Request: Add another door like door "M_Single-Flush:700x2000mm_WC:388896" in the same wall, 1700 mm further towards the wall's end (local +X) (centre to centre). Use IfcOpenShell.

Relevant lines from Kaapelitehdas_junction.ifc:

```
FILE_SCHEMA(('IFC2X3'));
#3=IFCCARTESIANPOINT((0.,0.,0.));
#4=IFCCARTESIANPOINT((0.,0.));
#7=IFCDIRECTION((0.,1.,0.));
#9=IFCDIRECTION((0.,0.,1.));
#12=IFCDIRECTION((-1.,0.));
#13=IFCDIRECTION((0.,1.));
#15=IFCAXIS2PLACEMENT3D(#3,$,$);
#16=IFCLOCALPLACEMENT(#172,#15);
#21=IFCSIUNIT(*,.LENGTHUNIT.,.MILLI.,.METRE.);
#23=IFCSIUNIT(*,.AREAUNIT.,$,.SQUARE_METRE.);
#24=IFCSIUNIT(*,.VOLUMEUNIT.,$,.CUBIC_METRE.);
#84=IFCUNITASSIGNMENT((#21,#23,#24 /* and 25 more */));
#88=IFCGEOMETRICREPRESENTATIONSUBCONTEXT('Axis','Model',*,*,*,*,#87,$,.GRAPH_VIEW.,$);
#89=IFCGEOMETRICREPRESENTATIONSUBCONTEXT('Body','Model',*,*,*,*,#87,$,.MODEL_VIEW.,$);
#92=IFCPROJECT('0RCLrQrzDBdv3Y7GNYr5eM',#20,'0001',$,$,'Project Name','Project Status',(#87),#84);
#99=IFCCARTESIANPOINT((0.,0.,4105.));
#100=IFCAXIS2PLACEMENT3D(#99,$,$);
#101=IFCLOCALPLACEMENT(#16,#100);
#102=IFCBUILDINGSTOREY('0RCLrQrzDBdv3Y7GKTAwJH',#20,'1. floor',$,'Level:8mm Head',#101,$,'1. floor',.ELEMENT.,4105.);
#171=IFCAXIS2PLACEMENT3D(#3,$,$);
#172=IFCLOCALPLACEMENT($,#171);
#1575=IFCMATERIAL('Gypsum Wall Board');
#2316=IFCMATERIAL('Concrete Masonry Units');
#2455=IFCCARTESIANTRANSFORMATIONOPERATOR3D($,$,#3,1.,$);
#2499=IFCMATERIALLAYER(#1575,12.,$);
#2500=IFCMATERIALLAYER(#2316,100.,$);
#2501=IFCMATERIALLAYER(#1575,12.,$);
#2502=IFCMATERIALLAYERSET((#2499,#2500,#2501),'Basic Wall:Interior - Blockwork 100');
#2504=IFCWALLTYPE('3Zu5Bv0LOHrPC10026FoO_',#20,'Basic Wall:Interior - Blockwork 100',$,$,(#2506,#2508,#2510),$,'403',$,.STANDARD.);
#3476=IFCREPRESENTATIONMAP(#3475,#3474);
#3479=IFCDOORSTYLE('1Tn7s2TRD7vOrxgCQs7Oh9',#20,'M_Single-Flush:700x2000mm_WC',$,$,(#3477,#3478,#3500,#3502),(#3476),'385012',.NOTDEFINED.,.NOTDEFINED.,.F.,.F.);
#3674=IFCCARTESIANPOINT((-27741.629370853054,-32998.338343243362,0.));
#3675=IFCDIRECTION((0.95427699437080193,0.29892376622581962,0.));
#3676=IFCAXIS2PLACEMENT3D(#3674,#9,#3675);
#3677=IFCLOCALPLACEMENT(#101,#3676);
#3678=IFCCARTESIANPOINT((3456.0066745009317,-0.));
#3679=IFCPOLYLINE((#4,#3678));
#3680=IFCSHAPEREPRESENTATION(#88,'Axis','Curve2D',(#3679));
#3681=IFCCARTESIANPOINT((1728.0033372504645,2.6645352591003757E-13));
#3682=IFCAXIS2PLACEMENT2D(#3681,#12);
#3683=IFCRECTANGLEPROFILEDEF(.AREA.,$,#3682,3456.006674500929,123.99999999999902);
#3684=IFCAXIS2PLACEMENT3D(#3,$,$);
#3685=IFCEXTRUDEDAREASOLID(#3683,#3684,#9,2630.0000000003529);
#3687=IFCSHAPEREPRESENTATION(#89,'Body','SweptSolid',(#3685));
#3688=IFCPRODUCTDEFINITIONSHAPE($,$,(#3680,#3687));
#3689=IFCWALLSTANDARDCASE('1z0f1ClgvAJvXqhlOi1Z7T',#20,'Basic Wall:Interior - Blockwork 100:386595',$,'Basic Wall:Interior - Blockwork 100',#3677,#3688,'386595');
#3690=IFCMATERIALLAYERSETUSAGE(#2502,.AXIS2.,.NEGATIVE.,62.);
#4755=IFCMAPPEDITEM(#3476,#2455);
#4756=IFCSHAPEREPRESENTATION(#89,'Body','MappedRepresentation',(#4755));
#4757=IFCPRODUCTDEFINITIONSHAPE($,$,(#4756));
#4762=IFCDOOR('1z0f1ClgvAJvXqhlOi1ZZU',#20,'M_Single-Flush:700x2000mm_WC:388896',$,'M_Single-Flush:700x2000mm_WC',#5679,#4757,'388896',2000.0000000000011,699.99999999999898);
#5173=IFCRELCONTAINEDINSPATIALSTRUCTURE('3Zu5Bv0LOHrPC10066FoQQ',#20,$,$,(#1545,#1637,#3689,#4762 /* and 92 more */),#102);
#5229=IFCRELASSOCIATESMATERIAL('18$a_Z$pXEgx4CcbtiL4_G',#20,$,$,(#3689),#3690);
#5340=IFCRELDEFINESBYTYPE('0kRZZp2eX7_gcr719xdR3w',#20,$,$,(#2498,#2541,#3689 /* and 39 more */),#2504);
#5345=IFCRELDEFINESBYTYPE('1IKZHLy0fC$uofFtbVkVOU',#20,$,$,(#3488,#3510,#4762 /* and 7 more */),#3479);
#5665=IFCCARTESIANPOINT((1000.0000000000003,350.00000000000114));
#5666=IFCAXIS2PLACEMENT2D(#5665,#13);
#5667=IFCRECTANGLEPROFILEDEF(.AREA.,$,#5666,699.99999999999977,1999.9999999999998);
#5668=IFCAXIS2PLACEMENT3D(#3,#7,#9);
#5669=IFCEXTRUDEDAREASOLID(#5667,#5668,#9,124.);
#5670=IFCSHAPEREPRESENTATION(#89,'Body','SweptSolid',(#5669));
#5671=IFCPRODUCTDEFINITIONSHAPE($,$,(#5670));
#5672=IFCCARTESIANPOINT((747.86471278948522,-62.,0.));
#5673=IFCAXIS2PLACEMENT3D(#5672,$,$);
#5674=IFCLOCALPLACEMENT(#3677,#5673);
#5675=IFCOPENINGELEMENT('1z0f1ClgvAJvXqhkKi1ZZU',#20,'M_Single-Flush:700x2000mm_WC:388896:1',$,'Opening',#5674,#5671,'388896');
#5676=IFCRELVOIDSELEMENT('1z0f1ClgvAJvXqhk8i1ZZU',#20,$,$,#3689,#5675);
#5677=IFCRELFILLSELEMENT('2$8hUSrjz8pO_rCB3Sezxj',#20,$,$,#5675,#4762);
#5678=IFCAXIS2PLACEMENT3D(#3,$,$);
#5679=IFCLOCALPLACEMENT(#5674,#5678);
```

```python
import ifcopenshell
import ifcopenshell.api.feature
import ifcopenshell.api.geometry
import ifcopenshell.api.root
import ifcopenshell.geom
import ifcopenshell.util.element
import ifcopenshell.util.placement
import ifcopenshell.util.shape

model = ifcopenshell.open("Kaapelitehdas_junction.ifc")
settings = ifcopenshell.geom.settings()


def volume(element):
    """Net volume in cubic metres, openings subtracted."""
    shape = ifcopenshell.geom.create_shape(settings, element)
    return ifcopenshell.util.shape.get_volume(shape.geometry)


def reuse_history(source, copy):
    """copy_class also copies each property set's owner history, people and application; keep the originals."""
    for rel in copy.IsDefinedBy:
        if rel.is_a("IfcRelDefinesByProperties") and (history := rel.RelatingPropertyDefinition.OwnerHistory):
            rel.RelatingPropertyDefinition.OwnerHistory = source.OwnerHistory
            ifcopenshell.util.element.remove_deep2(model, history)


door = model.by_guid("1z0f1ClgvAJvXqhlOi1ZZU")
opening = door.FillsVoids[0].RelatingOpeningElement
wall = opening.VoidsElements[0].RelatingBuildingElement
before = volume(wall)
shift = ifcopenshell.util.placement.get_local_placement(wall.ObjectPlacement)[:3, 0] * 1700.0

# copy_class copies the void relationship, type, container and properties, but no geometry.
new_opening = ifcopenshell.api.root.copy_class(model, product=opening)
new_opening.Representation = ifcopenshell.util.element.copy_deep(
    model, opening.Representation, exclude=["IfcGeometricRepresentationContext", "IfcRepresentationMap"]
)
new_opening.Name = "M_Single-Flush:700x2000mm_WC"
new_opening.Tag = None
new_door = ifcopenshell.api.root.copy_class(model, product=door)
new_door.Representation = ifcopenshell.util.element.copy_deep(
    model, door.Representation, exclude=["IfcGeometricRepresentationContext", "IfcRepresentationMap"]
)
new_door.Name = "M_Single-Flush:700x2000mm_WC"
new_door.Tag = None
reuse_history(door, new_door)
fills = ifcopenshell.api.feature.add_filling(model, opening=new_opening, element=new_door)
fills.OwnerHistory = new_door.OwnerHistory  # required in IFC2X3

for old, new in ((opening, new_opening), (door, new_door)):
    matrix = ifcopenshell.util.placement.get_local_placement(old.ObjectPlacement)
    matrix[:3, 3] += shift
    ifcopenshell.api.geometry.edit_object_placement(model, product=new, matrix=matrix, is_si=False)

after = volume(wall)

print(f"wall volume {before:.3f} -> {after:.3f} m3")

model.write("Kaapelitehdas_junction-out.ifc")
```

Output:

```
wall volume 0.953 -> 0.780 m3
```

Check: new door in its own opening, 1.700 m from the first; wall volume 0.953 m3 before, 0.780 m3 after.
